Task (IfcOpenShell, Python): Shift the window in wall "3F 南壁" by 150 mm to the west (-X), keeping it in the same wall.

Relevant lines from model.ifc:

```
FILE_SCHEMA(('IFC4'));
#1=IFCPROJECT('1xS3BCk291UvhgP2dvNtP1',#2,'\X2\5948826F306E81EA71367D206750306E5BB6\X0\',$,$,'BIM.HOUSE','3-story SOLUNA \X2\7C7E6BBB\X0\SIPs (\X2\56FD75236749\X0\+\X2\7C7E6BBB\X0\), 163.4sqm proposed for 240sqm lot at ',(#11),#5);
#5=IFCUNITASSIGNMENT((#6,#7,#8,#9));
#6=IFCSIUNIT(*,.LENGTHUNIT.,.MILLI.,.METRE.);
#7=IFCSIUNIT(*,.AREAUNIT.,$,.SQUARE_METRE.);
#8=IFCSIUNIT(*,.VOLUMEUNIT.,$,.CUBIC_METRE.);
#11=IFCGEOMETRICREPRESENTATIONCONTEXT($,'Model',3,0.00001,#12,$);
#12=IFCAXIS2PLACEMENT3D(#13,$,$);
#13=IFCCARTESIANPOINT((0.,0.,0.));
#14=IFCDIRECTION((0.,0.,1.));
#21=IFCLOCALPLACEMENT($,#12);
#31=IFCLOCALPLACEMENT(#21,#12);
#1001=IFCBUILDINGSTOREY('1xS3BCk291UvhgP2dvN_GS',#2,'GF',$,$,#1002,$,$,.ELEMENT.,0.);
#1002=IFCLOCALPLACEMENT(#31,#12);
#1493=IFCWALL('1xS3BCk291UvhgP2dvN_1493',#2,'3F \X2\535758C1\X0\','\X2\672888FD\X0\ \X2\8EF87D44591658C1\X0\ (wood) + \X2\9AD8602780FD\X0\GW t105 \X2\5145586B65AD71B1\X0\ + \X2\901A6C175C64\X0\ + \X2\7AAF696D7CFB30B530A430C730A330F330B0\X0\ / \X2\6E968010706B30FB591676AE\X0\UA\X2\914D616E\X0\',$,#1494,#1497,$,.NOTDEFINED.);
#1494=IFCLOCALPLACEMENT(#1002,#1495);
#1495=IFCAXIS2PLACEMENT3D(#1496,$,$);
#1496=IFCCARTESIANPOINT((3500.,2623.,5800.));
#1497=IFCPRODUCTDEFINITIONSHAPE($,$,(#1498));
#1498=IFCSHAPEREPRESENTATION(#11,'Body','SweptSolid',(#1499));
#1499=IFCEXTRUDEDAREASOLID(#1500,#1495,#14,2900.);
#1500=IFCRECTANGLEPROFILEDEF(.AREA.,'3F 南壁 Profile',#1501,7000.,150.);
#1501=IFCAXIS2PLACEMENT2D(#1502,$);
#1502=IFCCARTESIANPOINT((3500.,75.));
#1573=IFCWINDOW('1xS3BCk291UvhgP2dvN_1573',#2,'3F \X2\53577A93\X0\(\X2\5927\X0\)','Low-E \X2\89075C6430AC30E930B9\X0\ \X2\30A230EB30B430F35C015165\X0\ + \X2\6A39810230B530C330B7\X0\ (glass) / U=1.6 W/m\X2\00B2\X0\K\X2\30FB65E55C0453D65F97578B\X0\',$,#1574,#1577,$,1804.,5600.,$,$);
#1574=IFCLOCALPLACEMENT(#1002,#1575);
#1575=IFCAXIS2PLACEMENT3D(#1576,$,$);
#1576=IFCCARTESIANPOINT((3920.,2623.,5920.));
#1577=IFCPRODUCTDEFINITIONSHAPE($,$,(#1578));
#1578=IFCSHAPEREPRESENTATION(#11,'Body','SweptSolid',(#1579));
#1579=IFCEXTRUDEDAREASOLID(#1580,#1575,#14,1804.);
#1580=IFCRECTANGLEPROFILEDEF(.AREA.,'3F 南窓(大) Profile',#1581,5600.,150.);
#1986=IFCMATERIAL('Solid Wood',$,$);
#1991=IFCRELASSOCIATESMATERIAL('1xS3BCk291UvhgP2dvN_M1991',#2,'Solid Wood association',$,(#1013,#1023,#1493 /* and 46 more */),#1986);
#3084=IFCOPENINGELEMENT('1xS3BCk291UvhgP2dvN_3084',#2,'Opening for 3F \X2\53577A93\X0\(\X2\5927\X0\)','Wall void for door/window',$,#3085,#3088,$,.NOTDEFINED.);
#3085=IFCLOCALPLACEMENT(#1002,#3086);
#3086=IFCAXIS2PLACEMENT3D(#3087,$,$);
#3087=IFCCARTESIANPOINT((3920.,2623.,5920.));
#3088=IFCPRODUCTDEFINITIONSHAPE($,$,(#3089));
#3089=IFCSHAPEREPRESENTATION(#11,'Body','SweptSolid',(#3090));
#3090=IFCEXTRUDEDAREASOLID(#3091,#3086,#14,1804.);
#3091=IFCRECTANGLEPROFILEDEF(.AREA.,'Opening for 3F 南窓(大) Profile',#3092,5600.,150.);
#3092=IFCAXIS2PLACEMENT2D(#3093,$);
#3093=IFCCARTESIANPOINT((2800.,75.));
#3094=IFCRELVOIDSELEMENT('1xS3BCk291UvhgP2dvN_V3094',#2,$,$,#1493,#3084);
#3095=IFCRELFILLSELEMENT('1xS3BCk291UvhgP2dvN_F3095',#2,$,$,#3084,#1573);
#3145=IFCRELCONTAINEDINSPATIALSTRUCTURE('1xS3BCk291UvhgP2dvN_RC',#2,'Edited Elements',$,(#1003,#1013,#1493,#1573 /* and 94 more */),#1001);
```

```python
import ifcopenshell
import ifcopenshell.api.geometry
import ifcopenshell.util.placement

model = ifcopenshell.open("model.ifc")

window = model.by_guid("1xS3BCk291UvhgP2dvN_1573")
opening = window.FillsVoids[0].RelatingOpeningElement
wall = opening.VoidsElements[0].RelatingBuildingElement

wall_matrix = ifcopenshell.util.placement.get_local_placement(wall.ObjectPlacement)
shift = wall_matrix[:3, 0] * -150.0
before = ifcopenshell.util.placement.get_local_placement(window.ObjectPlacement)[:3, 3].copy()

# The window is not placed relative to its opening, so move both.
for product in (opening, window):
    matrix = ifcopenshell.util.placement.get_local_placement(product.ObjectPlacement)
    matrix[:3, 3] += shift
    ifcopenshell.api.geometry.edit_object_placement(model, product=product, matrix=matrix, is_si=False)

after = ifcopenshell.util.placement.get_local_placement(window.ObjectPlacement)[:3, 3]
print("window moved by", (after - before).round(3) + 0.0)

model.write("model-out.ifc")
```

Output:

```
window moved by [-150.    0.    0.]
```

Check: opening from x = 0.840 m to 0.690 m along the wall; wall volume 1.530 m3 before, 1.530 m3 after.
